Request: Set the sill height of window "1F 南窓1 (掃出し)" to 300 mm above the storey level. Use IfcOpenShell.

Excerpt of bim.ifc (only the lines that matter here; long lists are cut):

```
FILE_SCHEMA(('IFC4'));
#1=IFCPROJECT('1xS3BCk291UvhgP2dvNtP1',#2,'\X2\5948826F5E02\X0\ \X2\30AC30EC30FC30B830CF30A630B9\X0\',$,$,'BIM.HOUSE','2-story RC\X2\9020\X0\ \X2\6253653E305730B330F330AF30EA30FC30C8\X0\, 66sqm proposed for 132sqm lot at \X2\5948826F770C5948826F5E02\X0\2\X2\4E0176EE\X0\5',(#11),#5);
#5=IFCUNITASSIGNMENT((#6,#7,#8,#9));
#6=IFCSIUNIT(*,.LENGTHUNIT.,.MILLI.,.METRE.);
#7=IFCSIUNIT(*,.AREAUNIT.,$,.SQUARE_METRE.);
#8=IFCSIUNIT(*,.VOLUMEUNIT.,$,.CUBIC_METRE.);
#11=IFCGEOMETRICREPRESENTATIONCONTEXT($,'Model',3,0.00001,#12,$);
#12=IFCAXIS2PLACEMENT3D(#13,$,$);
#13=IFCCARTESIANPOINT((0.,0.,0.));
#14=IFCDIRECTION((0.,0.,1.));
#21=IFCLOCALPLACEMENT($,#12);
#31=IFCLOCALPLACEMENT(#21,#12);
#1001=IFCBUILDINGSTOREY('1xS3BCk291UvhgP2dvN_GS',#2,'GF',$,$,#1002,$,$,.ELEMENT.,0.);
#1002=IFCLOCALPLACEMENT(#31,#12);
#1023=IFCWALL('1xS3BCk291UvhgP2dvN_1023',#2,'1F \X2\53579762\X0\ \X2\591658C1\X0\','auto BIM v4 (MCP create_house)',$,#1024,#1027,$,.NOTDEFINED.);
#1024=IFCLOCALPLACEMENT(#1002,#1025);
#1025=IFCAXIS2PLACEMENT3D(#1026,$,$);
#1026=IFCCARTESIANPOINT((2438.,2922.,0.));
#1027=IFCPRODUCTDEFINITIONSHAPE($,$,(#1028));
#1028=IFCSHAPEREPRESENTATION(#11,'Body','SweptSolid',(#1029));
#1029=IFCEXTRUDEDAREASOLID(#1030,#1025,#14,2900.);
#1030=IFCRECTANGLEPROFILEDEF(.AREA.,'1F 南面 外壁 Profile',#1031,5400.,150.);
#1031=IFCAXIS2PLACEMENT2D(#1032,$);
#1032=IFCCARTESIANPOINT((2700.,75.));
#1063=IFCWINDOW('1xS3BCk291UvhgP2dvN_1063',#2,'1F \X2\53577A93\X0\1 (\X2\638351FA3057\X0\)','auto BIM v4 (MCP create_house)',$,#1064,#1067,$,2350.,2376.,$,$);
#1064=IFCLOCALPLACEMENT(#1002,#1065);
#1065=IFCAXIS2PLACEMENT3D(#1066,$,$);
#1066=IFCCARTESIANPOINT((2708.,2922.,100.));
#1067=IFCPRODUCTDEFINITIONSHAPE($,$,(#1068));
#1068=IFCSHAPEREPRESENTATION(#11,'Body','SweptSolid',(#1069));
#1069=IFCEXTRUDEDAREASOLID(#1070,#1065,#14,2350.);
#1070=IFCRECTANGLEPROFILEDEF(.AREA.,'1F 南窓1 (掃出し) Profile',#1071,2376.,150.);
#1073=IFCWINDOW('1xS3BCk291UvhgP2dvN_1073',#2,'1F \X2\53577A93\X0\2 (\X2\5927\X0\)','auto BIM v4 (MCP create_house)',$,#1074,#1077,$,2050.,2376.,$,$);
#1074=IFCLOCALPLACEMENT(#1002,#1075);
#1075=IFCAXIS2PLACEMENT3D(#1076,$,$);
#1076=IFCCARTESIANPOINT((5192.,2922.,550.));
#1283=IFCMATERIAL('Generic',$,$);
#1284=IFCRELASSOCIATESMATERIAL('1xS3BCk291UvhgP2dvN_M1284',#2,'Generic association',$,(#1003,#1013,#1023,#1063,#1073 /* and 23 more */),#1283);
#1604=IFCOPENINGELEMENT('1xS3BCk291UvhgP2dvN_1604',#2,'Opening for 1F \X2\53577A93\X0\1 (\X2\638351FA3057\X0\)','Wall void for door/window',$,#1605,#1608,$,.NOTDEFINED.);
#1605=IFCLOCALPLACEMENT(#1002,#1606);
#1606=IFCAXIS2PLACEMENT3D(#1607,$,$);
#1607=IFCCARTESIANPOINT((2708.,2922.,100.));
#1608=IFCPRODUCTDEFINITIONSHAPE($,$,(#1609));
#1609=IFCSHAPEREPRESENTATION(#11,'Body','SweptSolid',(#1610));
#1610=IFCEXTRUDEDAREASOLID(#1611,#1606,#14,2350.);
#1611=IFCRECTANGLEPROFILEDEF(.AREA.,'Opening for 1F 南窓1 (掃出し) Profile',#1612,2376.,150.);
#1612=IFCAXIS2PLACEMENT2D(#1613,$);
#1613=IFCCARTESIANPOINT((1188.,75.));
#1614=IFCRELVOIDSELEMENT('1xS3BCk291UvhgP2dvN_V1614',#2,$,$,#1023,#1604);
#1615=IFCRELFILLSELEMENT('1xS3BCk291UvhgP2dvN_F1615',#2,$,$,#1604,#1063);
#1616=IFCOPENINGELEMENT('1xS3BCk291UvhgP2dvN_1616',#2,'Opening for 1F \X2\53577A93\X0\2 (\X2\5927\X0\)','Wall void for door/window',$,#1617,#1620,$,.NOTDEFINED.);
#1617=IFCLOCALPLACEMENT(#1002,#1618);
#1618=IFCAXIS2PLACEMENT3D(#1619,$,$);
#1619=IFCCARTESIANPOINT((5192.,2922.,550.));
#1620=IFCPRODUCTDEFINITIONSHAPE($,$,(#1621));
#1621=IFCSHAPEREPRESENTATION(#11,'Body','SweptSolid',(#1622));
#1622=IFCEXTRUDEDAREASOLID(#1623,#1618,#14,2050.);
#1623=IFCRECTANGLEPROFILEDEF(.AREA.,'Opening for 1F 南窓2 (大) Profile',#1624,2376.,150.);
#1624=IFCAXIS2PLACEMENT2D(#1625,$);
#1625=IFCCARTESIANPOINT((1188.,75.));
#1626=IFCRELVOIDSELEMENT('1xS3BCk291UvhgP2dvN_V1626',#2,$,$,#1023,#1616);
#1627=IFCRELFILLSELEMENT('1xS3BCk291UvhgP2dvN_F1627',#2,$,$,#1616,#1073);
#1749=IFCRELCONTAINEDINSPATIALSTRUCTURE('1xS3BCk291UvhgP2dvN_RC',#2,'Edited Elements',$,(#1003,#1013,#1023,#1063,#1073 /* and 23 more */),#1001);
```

```python
import numpy as np
import ifcopenshell
import ifcopenshell.api.geometry
import ifcopenshell.geom
import ifcopenshell.util.element
import ifcopenshell.util.placement
import ifcopenshell.util.shape
import ifcopenshell.util.unit

model = ifcopenshell.open("bim.ifc")
unit_scale = ifcopenshell.util.unit.calculate_unit_scale(model)

window = model.by_id(1063)
opening = window.FillsVoids[0].RelatingOpeningElement
storey = ifcopenshell.util.element.get_container(window, ifc_class="IfcBuildingStorey")
level = ifcopenshell.util.placement.get_local_placement(storey.ObjectPlacement)[2, 3]

# The opening's origin need not be at the sill, so measure its lowest point.
shape = ifcopenshell.geom.create_shape(ifcopenshell.geom.settings(), opening)
bottom = ifcopenshell.util.shape.get_shape_bottom_elevation(shape, shape.geometry) / unit_scale
dz = level + 0.3 / unit_scale - bottom

shift = np.array([0.0, 0.0, dz])
# The window is not placed relative to its opening, so move both.
for product in (opening, window):
    matrix = ifcopenshell.util.placement.get_local_placement(product.ObjectPlacement)
    matrix[:3, 3] += shift
    ifcopenshell.api.geometry.edit_object_placement(model, product=product, matrix=matrix, is_si=False)

print(f"moved by {dz * unit_scale:+.3f} m")

model.write("bim_updated.ifc")
```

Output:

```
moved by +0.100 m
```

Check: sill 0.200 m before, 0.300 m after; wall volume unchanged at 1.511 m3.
